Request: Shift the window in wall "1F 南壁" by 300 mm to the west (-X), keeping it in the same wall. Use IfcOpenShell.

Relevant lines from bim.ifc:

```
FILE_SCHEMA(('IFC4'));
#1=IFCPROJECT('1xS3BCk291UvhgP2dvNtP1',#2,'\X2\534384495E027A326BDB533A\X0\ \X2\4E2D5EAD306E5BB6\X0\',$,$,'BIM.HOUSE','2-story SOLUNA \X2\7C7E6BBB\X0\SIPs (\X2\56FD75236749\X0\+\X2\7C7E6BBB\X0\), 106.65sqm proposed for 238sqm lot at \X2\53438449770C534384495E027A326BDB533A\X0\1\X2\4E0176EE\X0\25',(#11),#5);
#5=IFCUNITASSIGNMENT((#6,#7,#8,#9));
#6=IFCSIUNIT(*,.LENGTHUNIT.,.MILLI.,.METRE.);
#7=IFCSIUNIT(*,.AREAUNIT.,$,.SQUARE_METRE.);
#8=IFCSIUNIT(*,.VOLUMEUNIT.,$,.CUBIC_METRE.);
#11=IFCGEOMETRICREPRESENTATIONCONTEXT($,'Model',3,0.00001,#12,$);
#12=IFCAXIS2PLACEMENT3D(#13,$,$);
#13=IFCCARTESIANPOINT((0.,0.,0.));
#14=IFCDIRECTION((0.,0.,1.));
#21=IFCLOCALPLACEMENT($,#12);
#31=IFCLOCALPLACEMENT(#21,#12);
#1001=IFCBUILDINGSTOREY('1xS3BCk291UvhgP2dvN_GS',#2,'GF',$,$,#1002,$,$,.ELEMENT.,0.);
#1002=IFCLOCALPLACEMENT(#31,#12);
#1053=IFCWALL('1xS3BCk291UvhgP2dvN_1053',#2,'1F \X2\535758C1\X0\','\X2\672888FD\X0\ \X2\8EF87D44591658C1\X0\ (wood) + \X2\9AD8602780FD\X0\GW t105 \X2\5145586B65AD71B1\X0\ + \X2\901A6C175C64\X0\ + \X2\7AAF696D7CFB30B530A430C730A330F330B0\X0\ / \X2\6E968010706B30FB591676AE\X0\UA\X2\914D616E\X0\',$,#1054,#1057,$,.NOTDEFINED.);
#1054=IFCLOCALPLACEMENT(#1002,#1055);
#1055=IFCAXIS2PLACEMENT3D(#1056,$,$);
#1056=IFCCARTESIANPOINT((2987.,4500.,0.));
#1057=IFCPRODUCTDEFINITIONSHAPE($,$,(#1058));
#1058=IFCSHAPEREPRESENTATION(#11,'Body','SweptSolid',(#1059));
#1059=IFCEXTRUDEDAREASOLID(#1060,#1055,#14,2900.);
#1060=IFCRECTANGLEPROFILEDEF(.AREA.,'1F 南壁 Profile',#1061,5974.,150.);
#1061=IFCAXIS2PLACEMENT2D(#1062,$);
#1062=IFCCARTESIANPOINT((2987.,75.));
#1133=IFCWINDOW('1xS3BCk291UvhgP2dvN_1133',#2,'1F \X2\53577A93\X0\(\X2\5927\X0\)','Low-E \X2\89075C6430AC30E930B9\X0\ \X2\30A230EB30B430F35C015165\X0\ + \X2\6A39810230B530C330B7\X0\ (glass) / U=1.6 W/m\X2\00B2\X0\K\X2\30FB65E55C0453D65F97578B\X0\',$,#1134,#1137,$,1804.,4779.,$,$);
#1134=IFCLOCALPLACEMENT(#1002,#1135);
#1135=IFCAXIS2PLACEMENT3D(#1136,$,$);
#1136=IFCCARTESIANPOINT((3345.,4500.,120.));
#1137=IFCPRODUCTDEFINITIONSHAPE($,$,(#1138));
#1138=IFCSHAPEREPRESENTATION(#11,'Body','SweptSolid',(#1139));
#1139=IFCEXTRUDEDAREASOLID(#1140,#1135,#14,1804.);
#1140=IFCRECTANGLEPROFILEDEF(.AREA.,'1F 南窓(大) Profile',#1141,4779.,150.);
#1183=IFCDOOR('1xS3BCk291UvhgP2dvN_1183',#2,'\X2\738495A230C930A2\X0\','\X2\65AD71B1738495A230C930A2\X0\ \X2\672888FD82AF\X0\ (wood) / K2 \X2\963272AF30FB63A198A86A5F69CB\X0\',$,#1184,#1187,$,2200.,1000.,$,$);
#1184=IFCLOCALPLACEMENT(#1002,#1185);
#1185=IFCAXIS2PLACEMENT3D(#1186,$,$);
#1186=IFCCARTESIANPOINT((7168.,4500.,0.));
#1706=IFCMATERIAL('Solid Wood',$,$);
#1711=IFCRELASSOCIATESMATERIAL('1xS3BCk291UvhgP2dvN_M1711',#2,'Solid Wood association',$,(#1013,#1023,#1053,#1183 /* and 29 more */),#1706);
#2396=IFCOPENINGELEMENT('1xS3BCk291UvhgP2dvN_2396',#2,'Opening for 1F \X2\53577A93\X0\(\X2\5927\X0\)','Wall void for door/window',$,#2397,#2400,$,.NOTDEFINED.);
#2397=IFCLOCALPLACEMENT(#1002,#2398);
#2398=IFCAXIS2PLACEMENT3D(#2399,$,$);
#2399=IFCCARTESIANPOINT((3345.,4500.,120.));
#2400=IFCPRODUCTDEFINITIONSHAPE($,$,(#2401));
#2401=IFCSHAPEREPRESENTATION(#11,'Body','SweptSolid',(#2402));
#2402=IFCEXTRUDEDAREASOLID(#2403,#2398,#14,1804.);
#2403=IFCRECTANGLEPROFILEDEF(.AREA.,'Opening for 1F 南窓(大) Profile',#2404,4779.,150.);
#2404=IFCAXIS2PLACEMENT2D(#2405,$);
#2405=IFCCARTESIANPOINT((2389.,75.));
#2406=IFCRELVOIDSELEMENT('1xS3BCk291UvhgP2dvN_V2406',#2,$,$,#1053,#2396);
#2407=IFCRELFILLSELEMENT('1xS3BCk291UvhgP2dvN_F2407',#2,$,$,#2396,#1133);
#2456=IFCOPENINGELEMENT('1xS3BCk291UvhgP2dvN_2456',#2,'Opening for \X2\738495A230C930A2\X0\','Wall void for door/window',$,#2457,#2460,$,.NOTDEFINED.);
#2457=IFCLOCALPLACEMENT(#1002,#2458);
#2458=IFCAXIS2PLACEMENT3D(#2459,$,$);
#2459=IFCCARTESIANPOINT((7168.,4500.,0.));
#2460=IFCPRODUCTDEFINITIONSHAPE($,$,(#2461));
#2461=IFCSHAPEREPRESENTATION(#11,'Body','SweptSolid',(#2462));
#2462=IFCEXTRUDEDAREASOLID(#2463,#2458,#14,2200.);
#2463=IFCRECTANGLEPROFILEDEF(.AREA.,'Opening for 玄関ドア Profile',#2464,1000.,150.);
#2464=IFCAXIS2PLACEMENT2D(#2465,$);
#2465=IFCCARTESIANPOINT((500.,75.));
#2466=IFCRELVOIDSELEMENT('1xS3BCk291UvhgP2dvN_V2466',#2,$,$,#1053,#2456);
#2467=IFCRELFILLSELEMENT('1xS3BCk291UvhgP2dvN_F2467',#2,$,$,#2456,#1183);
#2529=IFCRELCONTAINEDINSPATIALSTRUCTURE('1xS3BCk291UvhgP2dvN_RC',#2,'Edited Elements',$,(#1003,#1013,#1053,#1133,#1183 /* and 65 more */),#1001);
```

```python
import ifcopenshell
import ifcopenshell.api.geometry
import ifcopenshell.util.placement

model = ifcopenshell.open("bim.ifc")

window = model.by_guid("1xS3BCk291UvhgP2dvN_1133")
opening = window.FillsVoids[0].RelatingOpeningElement
wall = opening.VoidsElements[0].RelatingBuildingElement

wall_matrix = ifcopenshell.util.placement.get_local_placement(wall.ObjectPlacement)
shift = wall_matrix[:3, 0] * -300.0
before = ifcopenshell.util.placement.get_local_placement(window.ObjectPlacement)[:3, 3].copy()

# The window is not placed relative to its opening, so move both.
for product in (opening, window):
    matrix = ifcopenshell.util.placement.get_local_placement(product.ObjectPlacement)
    matrix[:3, 3] += shift
    ifcopenshell.api.geometry.edit_object_placement(model, product=product, matrix=matrix, is_si=False)

after = ifcopenshell.util.placement.get_local_placement(window.ObjectPlacement)[:3, 3]
print("window moved by", (after - before).round(3) + 0.0)

model.write("bim_v2.ifc")
```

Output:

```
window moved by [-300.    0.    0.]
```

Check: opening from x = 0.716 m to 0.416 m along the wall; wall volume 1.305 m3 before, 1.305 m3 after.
